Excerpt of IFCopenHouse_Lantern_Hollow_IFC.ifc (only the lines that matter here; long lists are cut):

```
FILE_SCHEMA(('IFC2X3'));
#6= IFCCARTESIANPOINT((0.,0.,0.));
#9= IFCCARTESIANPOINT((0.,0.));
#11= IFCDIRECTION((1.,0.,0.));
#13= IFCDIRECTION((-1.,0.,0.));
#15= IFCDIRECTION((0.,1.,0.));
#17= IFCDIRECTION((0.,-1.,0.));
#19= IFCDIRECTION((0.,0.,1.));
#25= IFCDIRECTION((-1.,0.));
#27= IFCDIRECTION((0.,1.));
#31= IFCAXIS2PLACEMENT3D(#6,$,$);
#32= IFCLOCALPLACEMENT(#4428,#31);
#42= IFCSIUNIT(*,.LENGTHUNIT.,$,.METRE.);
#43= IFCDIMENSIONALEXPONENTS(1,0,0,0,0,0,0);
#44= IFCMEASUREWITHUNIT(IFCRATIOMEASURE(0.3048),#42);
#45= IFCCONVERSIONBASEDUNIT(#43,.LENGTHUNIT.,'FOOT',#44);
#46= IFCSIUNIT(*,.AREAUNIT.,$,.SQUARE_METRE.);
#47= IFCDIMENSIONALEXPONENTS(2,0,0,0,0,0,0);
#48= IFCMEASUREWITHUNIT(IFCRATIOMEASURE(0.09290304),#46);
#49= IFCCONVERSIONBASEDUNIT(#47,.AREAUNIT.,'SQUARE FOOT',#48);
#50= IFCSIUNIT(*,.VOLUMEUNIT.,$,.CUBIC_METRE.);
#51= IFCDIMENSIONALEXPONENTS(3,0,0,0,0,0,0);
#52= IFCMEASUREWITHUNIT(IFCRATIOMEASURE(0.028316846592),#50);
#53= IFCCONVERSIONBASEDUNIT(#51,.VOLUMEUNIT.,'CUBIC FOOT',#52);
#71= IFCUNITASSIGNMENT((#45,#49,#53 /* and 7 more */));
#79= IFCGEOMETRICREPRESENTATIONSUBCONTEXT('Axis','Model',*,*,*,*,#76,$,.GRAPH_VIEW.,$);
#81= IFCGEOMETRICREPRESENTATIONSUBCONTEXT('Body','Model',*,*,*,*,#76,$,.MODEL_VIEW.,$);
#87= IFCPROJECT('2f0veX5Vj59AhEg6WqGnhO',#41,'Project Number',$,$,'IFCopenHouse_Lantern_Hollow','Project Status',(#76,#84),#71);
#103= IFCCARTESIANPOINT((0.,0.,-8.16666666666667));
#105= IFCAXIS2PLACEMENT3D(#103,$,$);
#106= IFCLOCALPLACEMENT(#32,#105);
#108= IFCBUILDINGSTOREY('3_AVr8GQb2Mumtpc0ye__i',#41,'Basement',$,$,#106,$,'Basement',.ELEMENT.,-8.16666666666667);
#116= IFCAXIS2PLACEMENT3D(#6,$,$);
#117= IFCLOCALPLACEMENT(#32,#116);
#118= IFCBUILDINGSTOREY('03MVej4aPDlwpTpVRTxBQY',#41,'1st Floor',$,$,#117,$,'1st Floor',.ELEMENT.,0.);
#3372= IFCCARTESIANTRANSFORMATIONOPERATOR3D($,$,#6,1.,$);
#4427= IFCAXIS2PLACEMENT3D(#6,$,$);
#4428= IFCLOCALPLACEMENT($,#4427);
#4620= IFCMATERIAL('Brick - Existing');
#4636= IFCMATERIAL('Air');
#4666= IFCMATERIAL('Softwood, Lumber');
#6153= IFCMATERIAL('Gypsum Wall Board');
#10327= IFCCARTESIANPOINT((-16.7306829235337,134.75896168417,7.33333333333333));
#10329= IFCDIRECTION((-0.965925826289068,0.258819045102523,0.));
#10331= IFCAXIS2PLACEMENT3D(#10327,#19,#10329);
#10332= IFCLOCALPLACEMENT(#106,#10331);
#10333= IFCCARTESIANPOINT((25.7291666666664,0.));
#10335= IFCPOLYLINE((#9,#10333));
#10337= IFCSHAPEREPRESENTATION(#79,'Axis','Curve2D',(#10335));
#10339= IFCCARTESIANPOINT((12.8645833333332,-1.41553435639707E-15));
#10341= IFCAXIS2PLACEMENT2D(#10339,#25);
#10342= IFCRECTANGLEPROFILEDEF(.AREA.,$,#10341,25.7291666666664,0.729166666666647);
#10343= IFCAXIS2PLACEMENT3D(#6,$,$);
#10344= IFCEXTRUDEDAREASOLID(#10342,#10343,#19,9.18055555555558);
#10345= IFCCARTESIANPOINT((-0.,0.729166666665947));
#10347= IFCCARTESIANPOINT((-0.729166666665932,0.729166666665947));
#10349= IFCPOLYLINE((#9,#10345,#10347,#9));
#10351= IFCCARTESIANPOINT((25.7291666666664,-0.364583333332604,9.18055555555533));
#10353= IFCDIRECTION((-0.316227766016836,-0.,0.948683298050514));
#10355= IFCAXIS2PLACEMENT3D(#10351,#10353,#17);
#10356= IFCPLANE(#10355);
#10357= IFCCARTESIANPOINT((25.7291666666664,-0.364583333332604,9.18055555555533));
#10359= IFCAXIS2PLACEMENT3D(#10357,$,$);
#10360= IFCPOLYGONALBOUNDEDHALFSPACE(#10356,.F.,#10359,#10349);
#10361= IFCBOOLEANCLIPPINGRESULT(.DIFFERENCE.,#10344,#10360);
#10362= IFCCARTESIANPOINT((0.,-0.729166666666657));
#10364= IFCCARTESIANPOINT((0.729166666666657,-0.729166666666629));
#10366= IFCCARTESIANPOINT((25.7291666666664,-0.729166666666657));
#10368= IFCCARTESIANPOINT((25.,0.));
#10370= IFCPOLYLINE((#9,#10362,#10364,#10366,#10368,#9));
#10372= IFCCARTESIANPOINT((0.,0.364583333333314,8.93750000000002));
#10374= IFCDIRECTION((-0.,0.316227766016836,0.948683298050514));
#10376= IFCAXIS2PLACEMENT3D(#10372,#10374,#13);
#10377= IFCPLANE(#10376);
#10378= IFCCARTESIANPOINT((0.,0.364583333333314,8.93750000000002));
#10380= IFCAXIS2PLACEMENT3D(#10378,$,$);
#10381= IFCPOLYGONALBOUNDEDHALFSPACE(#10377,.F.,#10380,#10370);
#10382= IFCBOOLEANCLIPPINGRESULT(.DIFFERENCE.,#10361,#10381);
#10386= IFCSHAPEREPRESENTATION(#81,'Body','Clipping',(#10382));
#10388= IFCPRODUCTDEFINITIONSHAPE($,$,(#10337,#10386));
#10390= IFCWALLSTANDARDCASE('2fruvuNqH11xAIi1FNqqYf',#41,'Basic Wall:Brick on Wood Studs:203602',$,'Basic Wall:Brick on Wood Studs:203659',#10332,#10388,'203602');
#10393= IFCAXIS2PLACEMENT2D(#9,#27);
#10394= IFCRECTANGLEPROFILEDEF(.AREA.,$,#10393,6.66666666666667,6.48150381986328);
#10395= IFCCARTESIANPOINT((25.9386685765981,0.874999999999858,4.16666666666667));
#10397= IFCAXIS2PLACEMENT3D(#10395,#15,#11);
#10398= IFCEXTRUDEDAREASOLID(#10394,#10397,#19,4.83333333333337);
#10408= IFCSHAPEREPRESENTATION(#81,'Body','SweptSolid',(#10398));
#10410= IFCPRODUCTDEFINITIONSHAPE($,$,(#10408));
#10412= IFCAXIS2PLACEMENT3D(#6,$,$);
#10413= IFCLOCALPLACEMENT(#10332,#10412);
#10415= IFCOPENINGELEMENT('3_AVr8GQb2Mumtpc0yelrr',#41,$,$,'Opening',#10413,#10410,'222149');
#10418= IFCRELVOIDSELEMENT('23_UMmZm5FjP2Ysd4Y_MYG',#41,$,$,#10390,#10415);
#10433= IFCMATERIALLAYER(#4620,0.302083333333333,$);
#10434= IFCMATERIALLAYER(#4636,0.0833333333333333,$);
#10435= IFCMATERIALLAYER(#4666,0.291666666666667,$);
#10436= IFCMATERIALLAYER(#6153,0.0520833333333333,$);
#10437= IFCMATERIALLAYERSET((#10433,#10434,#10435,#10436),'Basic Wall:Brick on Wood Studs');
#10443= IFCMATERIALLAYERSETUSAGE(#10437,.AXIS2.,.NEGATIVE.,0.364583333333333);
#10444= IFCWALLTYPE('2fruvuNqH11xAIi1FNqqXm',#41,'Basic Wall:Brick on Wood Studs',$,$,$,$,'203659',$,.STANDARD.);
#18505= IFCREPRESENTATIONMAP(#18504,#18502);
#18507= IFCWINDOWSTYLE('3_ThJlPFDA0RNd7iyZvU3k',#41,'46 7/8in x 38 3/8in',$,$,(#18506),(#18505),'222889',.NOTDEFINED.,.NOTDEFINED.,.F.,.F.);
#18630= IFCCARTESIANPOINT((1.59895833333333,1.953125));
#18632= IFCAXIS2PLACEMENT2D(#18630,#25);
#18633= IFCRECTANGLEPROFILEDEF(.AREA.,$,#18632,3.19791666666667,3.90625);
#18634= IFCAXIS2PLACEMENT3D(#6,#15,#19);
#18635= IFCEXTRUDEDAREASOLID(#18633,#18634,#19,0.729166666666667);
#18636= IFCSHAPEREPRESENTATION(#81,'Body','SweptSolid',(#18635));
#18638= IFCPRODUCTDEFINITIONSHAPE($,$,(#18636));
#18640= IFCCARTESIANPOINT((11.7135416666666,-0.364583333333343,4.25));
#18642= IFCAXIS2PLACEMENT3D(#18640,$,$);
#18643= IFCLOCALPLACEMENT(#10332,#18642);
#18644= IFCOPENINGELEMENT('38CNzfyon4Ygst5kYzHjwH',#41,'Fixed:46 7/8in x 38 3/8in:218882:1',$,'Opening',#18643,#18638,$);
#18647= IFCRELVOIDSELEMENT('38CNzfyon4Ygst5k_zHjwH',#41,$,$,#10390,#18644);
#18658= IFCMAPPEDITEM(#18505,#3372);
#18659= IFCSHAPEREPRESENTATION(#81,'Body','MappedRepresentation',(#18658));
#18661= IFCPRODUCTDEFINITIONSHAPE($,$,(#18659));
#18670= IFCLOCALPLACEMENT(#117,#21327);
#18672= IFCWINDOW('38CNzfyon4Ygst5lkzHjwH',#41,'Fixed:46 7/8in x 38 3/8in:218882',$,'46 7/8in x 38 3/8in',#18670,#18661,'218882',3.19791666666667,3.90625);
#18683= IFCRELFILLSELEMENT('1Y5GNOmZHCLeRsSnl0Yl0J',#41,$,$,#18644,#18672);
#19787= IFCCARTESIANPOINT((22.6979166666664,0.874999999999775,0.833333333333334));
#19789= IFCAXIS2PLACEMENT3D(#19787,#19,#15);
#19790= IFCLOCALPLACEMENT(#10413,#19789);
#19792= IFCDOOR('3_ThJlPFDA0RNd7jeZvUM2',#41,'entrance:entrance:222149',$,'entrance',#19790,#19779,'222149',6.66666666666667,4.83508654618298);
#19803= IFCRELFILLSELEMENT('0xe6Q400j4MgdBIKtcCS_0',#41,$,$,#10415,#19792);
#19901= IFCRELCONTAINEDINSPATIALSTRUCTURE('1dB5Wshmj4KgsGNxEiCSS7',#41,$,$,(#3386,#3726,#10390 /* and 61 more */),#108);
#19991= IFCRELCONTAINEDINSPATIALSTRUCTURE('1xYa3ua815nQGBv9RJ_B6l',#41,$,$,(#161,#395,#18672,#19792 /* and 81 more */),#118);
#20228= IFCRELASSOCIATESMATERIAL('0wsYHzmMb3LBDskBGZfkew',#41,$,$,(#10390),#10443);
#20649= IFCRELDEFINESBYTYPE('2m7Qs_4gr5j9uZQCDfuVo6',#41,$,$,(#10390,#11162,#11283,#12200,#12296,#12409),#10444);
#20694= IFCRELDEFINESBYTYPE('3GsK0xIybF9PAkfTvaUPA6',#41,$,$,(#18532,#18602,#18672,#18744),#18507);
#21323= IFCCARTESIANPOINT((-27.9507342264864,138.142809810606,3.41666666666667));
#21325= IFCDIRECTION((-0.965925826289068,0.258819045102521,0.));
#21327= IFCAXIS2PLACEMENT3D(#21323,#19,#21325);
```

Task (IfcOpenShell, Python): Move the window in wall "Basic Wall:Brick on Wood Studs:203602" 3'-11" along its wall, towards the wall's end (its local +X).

```python
import ifcopenshell
import ifcopenshell.api.geometry
import ifcopenshell.util.placement
import ifcopenshell.util.unit

model = ifcopenshell.open("IFCopenHouse_Lantern_Hollow_IFC.ifc")
unit_scale = ifcopenshell.util.unit.calculate_unit_scale(model)

window = model.by_id(18672)
opening = window.FillsVoids[0].RelatingOpeningElement
wall = opening.VoidsElements[0].RelatingBuildingElement

wall_matrix = ifcopenshell.util.placement.get_local_placement(wall.ObjectPlacement)
shift = wall_matrix[:3, 0] * 47 * 0.0254 / unit_scale
before = ifcopenshell.util.placement.get_local_placement(window.ObjectPlacement)[:3, 3].copy()

# The window is not placed relative to its opening, so move both.
for product in (opening, window):
    matrix = ifcopenshell.util.placement.get_local_placement(product.ObjectPlacement)
    matrix[:3, 3] += shift
    ifcopenshell.api.geometry.edit_object_placement(model, product=product, matrix=matrix, is_si=False)

after = ifcopenshell.util.placement.get_local_placement(window.ObjectPlacement)[:3, 3]
print("window moved by", (after - before).round(3) + 0.0)

model.write("IFCopenHouse_Lantern_Hollow_IFC_edited.ifc")
```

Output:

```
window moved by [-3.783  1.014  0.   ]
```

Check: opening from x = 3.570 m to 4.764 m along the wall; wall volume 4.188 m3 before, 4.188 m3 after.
